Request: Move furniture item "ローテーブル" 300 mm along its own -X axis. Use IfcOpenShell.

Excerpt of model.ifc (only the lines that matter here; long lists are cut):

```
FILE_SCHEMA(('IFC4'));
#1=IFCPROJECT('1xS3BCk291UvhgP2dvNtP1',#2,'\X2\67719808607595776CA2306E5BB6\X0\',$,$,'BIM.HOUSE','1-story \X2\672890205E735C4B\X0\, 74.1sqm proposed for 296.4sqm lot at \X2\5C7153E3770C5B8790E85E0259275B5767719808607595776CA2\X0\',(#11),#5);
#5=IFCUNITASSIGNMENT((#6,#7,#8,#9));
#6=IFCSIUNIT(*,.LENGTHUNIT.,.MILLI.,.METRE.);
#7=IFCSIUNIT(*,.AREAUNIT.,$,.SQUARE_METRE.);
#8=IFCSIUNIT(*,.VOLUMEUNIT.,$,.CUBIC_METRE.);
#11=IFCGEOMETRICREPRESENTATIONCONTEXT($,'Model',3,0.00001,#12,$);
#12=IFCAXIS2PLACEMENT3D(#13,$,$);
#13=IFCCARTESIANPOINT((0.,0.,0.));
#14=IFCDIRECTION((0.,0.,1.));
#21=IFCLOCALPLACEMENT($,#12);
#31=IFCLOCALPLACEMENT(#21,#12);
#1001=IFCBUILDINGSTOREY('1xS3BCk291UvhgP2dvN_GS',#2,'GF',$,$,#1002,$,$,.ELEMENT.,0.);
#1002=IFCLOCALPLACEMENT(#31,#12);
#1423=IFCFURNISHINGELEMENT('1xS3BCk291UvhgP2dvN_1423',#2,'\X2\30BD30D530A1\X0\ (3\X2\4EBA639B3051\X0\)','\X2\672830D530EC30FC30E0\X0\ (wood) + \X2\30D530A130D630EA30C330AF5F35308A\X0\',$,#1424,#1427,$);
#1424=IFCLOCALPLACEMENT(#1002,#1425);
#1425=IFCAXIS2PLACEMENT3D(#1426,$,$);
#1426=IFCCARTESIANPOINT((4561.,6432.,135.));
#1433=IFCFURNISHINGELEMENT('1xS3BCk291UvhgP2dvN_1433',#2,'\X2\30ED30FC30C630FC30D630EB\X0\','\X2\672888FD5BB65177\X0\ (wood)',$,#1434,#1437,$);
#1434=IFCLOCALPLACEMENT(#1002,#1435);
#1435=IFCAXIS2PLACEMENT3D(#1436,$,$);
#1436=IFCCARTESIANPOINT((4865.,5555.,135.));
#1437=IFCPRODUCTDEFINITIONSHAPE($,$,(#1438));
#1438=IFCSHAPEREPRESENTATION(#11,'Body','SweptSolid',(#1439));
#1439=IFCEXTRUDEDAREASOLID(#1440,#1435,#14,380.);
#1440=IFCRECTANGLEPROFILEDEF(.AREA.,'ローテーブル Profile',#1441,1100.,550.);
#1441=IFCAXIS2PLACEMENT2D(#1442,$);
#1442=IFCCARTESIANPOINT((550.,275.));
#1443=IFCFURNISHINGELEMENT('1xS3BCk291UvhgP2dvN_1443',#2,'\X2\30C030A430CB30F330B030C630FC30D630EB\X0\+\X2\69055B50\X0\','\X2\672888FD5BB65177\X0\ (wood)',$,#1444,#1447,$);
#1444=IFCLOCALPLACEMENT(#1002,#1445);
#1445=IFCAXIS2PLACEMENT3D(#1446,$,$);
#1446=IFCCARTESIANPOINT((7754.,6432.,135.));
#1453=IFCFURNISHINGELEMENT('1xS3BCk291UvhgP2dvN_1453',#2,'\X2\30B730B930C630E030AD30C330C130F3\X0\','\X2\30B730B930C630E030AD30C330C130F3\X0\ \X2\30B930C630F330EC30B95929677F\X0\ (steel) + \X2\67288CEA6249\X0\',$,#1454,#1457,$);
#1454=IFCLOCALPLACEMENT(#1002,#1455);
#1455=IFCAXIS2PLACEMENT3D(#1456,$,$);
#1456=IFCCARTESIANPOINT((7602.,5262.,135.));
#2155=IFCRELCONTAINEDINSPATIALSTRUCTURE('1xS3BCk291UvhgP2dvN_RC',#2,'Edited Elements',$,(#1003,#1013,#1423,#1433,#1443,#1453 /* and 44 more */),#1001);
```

```python
import ifcopenshell
import ifcopenshell.api.geometry
import ifcopenshell.util.placement

model = ifcopenshell.open("model.ifc")

item = model.by_guid("1xS3BCk291UvhgP2dvN_1433")
matrix = ifcopenshell.util.placement.get_local_placement(item.ObjectPlacement)
matrix[:3, 3] -= matrix[:3, 0] * 300.0
ifcopenshell.api.geometry.edit_object_placement(model, product=item, matrix=matrix, is_si=False)

print(ifcopenshell.util.placement.get_local_placement(item.ObjectPlacement).round(3) + 0.0)

model.write("model_v2.ifc")
```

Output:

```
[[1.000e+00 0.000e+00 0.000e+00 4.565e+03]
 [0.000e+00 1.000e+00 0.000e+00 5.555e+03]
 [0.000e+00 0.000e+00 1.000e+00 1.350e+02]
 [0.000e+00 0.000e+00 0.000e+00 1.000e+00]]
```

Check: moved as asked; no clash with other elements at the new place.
